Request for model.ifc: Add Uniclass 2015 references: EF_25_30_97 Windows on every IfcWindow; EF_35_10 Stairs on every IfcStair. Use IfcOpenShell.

First a look at what the model holds.

```python
import ifcopenshell

model = ifcopenshell.open("model.ifc")
print(model.schema)
print("classifications:", [c.Name for c in model.by_type("IfcClassification")])
for ifc_class in ("IfcDoor", "IfcRoof", "IfcStair", "IfcWall", "IfcWindow"):
    print(ifc_class, len(model.by_type(ifc_class)))
```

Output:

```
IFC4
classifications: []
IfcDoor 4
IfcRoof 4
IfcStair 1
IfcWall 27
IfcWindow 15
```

```python
import ifcopenshell
import ifcopenshell.api.classification

model = ifcopenshell.open("model.ifc")

system = ifcopenshell.api.classification.add_classification(model, classification="Uniclass 2015")

codes = {
    "IfcWindow": ("EF_25_30_97", "Windows"),
    "IfcStair": ("EF_35_10", "Stairs"),
}
for ifc_class, (code, name) in codes.items():
    products = model.by_type(ifc_class)
    ifcopenshell.api.classification.add_reference(
        model, products=products, classification=system, identification=code, name=name
    )
    print(code, len(products))

model.write("model-out.ifc")
```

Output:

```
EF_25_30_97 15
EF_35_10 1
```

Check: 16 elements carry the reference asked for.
